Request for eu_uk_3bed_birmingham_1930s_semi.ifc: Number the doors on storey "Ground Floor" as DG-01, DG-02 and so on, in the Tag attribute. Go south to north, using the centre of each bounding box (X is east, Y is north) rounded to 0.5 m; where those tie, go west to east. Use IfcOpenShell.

First a look at what the model holds.

```python
import ifcopenshell
import ifcopenshell.util.element
import ifcopenshell.util.placement

model = ifcopenshell.open("eu_uk_3bed_birmingham_1930s_semi.ifc")
print(model.schema)
storey = next(s for s in model.by_type("IfcBuildingStorey") if s.Name == "Ground Floor")
doors = [e for e in ifcopenshell.util.element.get_decomposition(storey) if e.is_a("IfcDoor")]
for e in sorted(doors, key=lambda e: e.id()):
    origin = ifcopenshell.util.placement.get_local_placement(e.ObjectPlacement)[:3, 3]
    print(e.id(), e.Tag, e.Name, origin.round(2) + 0.0, sep=" | ")
```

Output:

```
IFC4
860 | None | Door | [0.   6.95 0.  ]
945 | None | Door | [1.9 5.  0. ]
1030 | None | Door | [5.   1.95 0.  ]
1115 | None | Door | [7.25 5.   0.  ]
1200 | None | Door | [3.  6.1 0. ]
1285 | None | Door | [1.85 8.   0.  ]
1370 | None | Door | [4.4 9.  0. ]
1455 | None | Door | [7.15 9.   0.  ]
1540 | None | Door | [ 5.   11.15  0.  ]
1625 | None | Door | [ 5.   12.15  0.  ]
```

```python
import ifcopenshell
import ifcopenshell.geom
import ifcopenshell.util.element
import ifcopenshell.util.shape

model = ifcopenshell.open("eu_uk_3bed_birmingham_1930s_semi.ifc")
settings = ifcopenshell.geom.settings()
settings.set("use-world-coords", True)


def centre(element):
    shape = ifcopenshell.geom.create_shape(settings, element)
    return ifcopenshell.util.shape.get_bbox_centroid(shape.geometry)


storey = next(s for s in model.by_type("IfcBuildingStorey") if s.Name == "Ground Floor")
doors = [e for e in ifcopenshell.util.element.get_decomposition(storey) if e.is_a("IfcDoor")]

# Insertion points can sit at a corner or the storey origin, so sort by the geometry (in metres).
centres = {e: centre(e) for e in doors}
doors.sort(key=lambda e: (round(centres[e][1] / 0.5), centres[e][0]))

for i, e in enumerate(doors, start=1):
    number = f"DG-{i:02d}"
    e.Tag = number
    print(e.id(), number)

model.write("eu_uk_3bed_birmingham_1930s_semi_rev.ifc")
```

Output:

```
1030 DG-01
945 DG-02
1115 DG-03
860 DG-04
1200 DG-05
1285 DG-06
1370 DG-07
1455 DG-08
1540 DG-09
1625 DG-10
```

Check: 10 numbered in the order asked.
